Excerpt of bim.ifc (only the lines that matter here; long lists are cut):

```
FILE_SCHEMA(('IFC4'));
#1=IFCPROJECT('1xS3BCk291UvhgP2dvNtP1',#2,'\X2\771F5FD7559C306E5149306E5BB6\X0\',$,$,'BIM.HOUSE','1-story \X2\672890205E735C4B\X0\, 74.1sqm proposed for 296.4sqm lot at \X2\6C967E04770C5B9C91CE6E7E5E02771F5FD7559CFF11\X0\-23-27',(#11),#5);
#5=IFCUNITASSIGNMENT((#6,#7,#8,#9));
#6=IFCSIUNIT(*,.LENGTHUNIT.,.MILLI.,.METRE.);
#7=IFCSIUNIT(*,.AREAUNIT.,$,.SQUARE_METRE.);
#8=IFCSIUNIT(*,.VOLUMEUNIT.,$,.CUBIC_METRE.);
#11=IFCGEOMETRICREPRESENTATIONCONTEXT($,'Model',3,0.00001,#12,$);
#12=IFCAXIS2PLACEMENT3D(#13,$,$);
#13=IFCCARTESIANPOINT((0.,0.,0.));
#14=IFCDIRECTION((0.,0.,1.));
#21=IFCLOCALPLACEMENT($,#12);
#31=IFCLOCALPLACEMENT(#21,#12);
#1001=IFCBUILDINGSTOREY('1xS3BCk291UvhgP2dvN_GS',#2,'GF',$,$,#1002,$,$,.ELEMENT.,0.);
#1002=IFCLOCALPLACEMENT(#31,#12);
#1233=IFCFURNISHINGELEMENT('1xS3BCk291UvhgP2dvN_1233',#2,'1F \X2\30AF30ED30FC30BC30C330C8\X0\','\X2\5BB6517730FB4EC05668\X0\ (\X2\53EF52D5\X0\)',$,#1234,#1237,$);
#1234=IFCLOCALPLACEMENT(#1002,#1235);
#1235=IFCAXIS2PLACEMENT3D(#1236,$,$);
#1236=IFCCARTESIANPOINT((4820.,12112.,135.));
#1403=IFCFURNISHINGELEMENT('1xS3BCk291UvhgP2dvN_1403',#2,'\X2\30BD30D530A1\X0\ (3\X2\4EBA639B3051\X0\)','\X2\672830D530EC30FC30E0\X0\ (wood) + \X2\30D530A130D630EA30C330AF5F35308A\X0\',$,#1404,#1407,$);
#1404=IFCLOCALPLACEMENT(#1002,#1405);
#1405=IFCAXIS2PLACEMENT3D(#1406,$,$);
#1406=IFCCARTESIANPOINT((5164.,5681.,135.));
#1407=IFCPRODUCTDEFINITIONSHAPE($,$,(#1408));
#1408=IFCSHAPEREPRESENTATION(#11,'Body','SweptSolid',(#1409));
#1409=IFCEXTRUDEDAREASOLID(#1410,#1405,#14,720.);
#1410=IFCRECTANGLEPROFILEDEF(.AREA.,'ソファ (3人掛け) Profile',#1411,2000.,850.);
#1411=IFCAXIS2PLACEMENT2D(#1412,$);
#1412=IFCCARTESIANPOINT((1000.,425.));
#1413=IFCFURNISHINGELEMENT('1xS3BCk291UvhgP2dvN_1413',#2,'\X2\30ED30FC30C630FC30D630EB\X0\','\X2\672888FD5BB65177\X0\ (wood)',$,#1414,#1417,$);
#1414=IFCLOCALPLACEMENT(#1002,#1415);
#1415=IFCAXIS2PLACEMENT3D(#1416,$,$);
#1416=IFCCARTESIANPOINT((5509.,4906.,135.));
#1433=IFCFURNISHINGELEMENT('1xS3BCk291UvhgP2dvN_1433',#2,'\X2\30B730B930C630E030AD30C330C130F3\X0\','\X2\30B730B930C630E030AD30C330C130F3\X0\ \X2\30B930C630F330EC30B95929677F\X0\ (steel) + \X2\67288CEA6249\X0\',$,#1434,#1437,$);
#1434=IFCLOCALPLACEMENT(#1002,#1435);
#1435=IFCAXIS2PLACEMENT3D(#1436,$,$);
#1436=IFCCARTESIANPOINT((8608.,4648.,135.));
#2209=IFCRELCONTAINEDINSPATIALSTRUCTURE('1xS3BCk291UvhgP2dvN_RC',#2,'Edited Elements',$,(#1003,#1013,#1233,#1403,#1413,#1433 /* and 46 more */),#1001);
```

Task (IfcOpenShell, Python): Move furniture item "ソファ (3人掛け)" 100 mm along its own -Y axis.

```python
import ifcopenshell
import ifcopenshell.api.geometry
import ifcopenshell.util.placement
import ifcopenshell.util.unit

model = ifcopenshell.open("bim.ifc")
unit_scale = ifcopenshell.util.unit.calculate_unit_scale(model)

item = model.by_guid("1xS3BCk291UvhgP2dvN_1403")
matrix = ifcopenshell.util.placement.get_local_placement(item.ObjectPlacement)
matrix[:3, 3] -= matrix[:3, 1] * 0.1 / unit_scale
ifcopenshell.api.geometry.edit_object_placement(model, product=item, matrix=matrix, is_si=False)

print(ifcopenshell.util.placement.get_local_placement(item.ObjectPlacement).round(3) + 0.0)

model.write("bim_updated.ifc")
```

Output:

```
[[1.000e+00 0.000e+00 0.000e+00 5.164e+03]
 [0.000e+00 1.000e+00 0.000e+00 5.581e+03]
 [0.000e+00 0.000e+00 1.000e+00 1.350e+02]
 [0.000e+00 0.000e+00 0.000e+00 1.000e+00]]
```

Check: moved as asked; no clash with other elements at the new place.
